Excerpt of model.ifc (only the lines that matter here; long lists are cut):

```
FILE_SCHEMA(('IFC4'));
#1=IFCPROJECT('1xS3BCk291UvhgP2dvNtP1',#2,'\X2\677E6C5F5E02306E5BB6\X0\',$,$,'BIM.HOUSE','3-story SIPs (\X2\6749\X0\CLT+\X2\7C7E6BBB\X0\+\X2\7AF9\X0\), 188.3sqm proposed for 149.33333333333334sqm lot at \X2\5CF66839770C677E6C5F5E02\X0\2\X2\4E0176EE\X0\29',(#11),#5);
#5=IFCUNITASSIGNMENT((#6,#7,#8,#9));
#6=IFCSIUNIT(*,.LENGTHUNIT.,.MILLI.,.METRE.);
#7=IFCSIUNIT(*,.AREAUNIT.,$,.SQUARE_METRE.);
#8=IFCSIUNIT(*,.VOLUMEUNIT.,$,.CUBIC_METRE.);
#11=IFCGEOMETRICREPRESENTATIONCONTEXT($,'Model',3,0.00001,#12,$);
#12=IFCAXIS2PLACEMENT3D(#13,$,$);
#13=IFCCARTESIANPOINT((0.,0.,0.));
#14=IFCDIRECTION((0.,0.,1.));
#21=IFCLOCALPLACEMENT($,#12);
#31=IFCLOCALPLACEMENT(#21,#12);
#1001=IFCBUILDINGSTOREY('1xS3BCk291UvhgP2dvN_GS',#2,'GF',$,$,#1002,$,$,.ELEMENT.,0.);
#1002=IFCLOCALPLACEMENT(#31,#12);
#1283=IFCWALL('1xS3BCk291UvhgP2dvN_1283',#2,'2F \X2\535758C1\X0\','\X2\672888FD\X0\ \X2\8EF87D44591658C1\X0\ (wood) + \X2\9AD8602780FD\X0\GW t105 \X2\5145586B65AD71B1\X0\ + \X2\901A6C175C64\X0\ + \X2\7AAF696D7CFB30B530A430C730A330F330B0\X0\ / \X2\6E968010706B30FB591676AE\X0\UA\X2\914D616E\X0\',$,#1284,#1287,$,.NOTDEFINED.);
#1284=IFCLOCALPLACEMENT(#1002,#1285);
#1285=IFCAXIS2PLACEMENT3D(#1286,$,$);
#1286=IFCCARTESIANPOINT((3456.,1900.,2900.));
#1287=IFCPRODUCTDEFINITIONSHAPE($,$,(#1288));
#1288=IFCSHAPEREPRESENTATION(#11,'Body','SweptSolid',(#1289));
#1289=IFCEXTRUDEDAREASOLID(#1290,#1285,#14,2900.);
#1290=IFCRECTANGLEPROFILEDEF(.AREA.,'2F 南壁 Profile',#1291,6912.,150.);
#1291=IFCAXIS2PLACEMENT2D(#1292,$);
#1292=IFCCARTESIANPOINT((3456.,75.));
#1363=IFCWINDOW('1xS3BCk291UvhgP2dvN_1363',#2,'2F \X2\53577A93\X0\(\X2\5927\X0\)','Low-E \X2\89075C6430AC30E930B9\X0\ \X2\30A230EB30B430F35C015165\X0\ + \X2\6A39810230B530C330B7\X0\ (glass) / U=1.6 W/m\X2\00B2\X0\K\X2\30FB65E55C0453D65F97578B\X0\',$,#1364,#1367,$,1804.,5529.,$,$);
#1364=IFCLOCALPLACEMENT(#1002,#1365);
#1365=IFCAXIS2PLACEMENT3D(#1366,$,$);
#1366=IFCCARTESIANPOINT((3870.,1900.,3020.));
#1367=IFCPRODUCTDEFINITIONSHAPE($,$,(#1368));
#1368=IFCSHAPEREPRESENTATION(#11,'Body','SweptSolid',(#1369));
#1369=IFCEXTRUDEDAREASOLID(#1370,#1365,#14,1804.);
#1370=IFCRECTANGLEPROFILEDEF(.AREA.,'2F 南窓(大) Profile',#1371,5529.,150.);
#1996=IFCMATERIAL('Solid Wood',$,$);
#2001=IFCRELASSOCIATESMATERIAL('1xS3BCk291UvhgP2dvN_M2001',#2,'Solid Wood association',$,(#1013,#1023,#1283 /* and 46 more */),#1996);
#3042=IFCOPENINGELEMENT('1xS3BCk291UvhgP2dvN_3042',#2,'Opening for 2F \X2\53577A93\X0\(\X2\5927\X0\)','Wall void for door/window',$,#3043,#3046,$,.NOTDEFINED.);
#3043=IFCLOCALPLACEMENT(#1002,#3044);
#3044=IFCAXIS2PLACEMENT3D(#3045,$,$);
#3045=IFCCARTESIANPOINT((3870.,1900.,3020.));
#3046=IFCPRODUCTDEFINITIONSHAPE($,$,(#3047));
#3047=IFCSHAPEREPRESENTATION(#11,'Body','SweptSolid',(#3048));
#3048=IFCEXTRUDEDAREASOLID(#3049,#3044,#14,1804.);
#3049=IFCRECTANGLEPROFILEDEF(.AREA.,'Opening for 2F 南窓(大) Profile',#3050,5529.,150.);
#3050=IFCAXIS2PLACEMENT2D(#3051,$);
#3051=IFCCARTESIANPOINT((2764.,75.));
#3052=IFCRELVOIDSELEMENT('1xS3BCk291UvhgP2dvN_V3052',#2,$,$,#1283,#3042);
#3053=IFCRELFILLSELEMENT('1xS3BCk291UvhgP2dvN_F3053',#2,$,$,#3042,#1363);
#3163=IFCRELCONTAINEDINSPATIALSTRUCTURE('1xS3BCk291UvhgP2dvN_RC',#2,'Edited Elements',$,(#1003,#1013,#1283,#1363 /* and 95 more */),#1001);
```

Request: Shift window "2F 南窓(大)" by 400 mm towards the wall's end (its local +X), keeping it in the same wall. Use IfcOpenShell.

```python
import ifcopenshell
import ifcopenshell.api.geometry
import ifcopenshell.util.placement
import ifcopenshell.util.unit

model = ifcopenshell.open("model.ifc")
unit_scale = ifcopenshell.util.unit.calculate_unit_scale(model)

window = model.by_id(1363)
opening = window.FillsVoids[0].RelatingOpeningElement
wall = opening.VoidsElements[0].RelatingBuildingElement

wall_matrix = ifcopenshell.util.placement.get_local_placement(wall.ObjectPlacement)
shift = wall_matrix[:3, 0] * 0.4 / unit_scale
before = ifcopenshell.util.placement.get_local_placement(window.ObjectPlacement)[:3, 3].copy()

# The window is not placed relative to its opening, so move both.
for product in (opening, window):
    matrix = ifcopenshell.util.placement.get_local_placement(product.ObjectPlacement)
    matrix[:3, 3] += shift
    ifcopenshell.api.geometry.edit_object_placement(model, product=product, matrix=matrix, is_si=False)

after = ifcopenshell.util.placement.get_local_placement(window.ObjectPlacement)[:3, 3]
print("window moved by", (after - before).round(3) + 0.0)

model.write("model_rev.ifc")
```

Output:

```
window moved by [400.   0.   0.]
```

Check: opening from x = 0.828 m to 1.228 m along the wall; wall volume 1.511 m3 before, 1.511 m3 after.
